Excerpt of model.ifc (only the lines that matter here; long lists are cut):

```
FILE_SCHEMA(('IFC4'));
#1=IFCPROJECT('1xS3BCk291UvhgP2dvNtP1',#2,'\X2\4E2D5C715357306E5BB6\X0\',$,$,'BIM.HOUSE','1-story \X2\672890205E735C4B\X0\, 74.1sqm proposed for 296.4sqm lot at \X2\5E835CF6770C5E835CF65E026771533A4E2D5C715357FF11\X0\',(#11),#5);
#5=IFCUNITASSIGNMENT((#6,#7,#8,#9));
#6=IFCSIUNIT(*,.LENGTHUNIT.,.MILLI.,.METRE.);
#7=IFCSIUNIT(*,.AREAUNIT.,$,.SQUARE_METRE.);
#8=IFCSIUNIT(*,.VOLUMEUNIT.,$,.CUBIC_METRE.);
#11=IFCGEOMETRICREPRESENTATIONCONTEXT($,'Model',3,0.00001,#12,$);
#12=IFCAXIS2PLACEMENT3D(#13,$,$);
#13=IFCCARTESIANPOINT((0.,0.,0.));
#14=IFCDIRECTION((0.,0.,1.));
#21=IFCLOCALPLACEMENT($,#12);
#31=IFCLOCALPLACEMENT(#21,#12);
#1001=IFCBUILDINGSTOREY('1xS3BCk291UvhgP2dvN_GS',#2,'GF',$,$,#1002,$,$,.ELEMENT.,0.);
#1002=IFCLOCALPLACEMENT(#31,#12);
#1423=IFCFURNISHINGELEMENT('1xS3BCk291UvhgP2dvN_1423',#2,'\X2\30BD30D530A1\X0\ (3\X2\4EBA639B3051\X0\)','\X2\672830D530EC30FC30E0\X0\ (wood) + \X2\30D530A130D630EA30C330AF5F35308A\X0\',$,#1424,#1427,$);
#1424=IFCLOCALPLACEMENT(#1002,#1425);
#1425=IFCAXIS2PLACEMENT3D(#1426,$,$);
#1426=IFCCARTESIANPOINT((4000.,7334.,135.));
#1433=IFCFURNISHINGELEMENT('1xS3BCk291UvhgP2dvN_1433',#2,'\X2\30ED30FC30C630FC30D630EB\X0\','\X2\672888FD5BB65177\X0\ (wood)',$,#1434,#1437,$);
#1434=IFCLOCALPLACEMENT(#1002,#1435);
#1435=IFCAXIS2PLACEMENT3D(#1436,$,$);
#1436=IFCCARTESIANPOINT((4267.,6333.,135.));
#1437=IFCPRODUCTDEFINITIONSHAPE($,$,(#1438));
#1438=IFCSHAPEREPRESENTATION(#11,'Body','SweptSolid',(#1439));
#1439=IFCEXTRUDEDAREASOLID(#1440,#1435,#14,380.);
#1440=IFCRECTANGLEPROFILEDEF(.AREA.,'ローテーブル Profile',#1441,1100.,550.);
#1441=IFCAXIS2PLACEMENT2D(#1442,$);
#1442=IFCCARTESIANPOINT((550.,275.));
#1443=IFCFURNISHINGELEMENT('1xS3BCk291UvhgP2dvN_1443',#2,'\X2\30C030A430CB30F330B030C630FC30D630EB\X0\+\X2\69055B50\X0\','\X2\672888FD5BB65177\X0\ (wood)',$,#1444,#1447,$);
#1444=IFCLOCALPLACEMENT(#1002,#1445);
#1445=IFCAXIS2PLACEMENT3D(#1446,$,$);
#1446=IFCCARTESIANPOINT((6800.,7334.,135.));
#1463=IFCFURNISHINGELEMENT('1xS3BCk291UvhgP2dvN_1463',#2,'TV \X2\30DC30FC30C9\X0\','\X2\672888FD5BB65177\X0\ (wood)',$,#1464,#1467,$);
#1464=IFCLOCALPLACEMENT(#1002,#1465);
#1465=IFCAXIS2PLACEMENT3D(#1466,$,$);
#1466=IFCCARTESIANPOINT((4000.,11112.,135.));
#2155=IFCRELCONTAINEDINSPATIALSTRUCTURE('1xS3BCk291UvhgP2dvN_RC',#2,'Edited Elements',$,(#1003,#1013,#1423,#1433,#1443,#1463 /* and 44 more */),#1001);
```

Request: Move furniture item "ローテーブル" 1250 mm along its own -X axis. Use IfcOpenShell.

```python
import ifcopenshell
import ifcopenshell.api.geometry
import ifcopenshell.util.placement
import ifcopenshell.util.unit

model = ifcopenshell.open("model.ifc")
unit_scale = ifcopenshell.util.unit.calculate_unit_scale(model)

item = model.by_guid("1xS3BCk291UvhgP2dvN_1433")
matrix = ifcopenshell.util.placement.get_local_placement(item.ObjectPlacement)
matrix[:3, 3] -= matrix[:3, 0] * 1.25 / unit_scale
ifcopenshell.api.geometry.edit_object_placement(model, product=item, matrix=matrix, is_si=False)

print(ifcopenshell.util.placement.get_local_placement(item.ObjectPlacement).round(3) + 0.0)

model.write("model_rev.ifc")
```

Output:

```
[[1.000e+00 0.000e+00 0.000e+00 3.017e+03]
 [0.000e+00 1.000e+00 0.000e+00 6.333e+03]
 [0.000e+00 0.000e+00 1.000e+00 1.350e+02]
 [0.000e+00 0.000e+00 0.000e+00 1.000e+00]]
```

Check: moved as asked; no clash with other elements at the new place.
